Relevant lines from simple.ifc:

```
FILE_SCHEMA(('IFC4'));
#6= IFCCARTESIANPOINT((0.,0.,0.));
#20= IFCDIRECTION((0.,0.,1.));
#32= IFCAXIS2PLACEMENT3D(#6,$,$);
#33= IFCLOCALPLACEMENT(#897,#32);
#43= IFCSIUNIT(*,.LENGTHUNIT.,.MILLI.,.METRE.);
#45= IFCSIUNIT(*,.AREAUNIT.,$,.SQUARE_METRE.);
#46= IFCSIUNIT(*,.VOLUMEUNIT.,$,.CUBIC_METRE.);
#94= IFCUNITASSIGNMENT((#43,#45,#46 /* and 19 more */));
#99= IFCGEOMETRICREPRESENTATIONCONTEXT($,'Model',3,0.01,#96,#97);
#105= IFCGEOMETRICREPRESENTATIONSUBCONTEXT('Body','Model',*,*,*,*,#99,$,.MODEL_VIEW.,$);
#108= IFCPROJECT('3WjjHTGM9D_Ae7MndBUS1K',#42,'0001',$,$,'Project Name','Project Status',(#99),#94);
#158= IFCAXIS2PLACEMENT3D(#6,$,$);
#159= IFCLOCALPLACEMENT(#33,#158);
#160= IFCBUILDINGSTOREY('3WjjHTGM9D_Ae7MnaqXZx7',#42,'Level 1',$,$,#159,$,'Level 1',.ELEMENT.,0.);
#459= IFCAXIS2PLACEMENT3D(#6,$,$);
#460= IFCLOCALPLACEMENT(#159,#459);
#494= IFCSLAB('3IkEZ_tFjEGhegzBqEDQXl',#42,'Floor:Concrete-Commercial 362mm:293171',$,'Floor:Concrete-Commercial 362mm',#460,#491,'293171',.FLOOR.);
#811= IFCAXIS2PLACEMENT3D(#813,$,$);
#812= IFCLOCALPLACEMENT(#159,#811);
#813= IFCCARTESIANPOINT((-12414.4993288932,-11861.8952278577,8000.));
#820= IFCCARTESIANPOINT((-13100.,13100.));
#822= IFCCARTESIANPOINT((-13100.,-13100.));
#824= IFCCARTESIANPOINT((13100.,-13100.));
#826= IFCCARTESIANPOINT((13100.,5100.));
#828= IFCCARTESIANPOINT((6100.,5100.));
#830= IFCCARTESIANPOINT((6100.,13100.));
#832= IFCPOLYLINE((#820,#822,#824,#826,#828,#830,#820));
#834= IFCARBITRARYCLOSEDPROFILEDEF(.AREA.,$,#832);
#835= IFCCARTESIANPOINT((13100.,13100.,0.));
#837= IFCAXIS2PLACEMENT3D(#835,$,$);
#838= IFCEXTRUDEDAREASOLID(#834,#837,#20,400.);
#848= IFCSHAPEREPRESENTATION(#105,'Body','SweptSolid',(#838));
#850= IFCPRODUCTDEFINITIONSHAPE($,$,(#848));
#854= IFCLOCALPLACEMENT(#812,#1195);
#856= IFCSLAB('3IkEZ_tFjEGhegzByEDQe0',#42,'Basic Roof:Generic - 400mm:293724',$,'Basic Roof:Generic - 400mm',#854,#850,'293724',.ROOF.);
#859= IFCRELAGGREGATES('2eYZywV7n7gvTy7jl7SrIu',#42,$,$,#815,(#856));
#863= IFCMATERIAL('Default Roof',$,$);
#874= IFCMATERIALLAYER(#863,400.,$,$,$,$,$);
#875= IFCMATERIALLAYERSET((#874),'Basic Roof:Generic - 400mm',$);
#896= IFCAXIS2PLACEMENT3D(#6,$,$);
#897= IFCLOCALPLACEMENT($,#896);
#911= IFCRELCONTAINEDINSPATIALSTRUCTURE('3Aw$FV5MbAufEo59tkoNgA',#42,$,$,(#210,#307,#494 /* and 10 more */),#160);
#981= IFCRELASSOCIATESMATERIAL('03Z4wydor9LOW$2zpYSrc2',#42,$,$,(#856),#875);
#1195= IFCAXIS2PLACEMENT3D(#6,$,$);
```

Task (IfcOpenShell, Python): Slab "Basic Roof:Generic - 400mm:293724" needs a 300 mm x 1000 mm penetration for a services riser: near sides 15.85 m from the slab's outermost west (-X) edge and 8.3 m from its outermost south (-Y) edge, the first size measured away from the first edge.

```python
import numpy as np
import ifcopenshell
import ifcopenshell.api.feature
import ifcopenshell.api.geometry
import ifcopenshell.api.root
import ifcopenshell.geom
import ifcopenshell.util.placement
import ifcopenshell.util.representation
import ifcopenshell.util.shape
import ifcopenshell.util.unit

model = ifcopenshell.open("simple.ifc")
unit_scale = ifcopenshell.util.unit.calculate_unit_scale(model)
settings = ifcopenshell.geom.settings()


def volume(element):
    """Net volume in cubic metres, openings subtracted."""
    shape = ifcopenshell.geom.create_shape(settings, element)
    return ifcopenshell.util.shape.get_volume(shape.geometry)


slab = model.by_guid("3IkEZ_tFjEGhegzByEDQe0")
before = volume(slab)

# Extent in the slab's own axes, in metres. The edges named are its -X and -Y sides.
slab_shape = ifcopenshell.geom.create_shape(settings, slab)
vertices = ifcopenshell.util.shape.get_vertices(slab_shape.geometry)
x_min, y_min, bottom = vertices.min(axis=0)
top = vertices[:, 2].max()

opening = ifcopenshell.api.root.create_entity(model, ifc_class="IfcOpeningElement", name="Services riser opening", predefined_type="OPENING")
context = ifcopenshell.util.representation.get_context(model, "Model", "Body", "MODEL_VIEW")
width, depth = 0.3, 1
outline = [(0.0, 0.0), (width, 0.0), (width, depth), (0.0, depth), (0.0, 0.0)]
# Overshoot both faces by 50 mm so the cut is clean.
shape = ifcopenshell.api.geometry.add_slab_representation(
    model, context=context, depth=top - bottom + 0.1, polyline=outline
)
ifcopenshell.api.geometry.assign_representation(model, product=opening, representation=shape)

matrix = ifcopenshell.util.placement.get_local_placement(slab.ObjectPlacement)
matrix[:, 3] = matrix @ np.append(np.array([x_min + 15.85, y_min + 8.3, bottom - 0.05]) / unit_scale, 1.0)
ifcopenshell.api.geometry.edit_object_placement(model, product=opening, matrix=matrix, is_si=False)
ifcopenshell.api.feature.add_feature(model, feature=opening, element=slab)

after = volume(slab)

print(f"slab volume {before:.3f} -> {after:.3f} m3")

model.write("simple-out.ifc")
```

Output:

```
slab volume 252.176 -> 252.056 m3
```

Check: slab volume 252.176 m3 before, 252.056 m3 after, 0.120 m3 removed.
